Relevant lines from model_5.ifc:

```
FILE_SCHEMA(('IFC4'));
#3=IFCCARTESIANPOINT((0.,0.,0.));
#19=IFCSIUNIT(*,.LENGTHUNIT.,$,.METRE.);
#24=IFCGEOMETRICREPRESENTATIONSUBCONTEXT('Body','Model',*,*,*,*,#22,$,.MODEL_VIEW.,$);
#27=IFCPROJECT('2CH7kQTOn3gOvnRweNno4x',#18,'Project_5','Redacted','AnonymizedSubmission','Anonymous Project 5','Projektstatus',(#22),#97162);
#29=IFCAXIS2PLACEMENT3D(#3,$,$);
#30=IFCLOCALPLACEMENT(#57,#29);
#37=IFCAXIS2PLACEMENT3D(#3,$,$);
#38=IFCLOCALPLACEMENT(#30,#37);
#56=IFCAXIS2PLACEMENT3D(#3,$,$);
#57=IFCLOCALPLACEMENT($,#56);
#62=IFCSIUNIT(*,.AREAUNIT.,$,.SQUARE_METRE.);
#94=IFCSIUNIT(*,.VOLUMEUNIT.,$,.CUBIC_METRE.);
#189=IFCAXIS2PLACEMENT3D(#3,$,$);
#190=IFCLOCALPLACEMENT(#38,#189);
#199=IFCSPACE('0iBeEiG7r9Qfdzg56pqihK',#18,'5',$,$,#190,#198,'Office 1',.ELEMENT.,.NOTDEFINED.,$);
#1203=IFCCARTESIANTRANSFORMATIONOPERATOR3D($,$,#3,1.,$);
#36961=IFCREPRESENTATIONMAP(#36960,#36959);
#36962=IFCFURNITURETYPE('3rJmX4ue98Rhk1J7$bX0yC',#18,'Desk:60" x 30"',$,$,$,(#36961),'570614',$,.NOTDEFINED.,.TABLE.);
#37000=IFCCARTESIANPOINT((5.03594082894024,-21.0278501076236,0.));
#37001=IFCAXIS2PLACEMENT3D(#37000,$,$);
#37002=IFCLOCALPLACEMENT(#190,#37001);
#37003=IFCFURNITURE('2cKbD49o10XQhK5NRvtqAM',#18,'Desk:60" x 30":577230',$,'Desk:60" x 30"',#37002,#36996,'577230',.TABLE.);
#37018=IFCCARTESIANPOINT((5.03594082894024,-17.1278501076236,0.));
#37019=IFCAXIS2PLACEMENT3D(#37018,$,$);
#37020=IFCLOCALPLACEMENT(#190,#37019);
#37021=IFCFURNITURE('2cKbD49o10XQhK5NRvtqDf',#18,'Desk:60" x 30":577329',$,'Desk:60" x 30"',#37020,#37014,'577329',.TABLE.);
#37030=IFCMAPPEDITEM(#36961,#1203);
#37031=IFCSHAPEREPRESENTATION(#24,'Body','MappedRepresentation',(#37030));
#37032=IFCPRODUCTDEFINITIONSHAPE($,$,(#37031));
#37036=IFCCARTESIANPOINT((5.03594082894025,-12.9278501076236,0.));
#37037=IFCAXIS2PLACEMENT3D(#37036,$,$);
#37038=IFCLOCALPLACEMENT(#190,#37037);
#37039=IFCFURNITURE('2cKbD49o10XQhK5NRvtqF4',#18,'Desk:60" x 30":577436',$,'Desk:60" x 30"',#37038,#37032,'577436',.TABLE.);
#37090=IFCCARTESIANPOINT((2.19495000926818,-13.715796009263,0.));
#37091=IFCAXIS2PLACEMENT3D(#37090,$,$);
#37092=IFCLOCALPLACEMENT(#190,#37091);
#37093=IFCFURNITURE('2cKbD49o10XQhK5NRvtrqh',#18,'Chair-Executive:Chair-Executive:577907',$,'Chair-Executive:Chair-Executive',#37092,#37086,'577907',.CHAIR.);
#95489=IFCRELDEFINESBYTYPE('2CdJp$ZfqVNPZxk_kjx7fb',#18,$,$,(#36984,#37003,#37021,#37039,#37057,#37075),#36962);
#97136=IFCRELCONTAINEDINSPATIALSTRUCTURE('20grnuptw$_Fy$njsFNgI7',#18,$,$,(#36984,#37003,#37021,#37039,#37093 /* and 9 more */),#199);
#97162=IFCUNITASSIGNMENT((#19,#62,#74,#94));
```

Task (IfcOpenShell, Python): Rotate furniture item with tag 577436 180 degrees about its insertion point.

```python
import ifcopenshell
import ifcopenshell.api.geometry
import ifcopenshell.util.placement

model = ifcopenshell.open("model_5.ifc")

item = model.by_guid("2cKbD49o10XQhK5NRvtqF4")
matrix = ifcopenshell.util.placement.get_local_placement(item.ObjectPlacement)
matrix = matrix @ ifcopenshell.util.placement.rotation(180, "Z")
ifcopenshell.api.geometry.edit_object_placement(model, product=item, matrix=matrix, is_si=False)

print(ifcopenshell.util.placement.get_local_placement(item.ObjectPlacement).round(3) + 0.0)

model.write("model_5-out.ifc")
```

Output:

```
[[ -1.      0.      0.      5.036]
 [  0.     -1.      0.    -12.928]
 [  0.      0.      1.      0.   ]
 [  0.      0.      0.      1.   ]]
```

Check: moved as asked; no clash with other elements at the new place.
